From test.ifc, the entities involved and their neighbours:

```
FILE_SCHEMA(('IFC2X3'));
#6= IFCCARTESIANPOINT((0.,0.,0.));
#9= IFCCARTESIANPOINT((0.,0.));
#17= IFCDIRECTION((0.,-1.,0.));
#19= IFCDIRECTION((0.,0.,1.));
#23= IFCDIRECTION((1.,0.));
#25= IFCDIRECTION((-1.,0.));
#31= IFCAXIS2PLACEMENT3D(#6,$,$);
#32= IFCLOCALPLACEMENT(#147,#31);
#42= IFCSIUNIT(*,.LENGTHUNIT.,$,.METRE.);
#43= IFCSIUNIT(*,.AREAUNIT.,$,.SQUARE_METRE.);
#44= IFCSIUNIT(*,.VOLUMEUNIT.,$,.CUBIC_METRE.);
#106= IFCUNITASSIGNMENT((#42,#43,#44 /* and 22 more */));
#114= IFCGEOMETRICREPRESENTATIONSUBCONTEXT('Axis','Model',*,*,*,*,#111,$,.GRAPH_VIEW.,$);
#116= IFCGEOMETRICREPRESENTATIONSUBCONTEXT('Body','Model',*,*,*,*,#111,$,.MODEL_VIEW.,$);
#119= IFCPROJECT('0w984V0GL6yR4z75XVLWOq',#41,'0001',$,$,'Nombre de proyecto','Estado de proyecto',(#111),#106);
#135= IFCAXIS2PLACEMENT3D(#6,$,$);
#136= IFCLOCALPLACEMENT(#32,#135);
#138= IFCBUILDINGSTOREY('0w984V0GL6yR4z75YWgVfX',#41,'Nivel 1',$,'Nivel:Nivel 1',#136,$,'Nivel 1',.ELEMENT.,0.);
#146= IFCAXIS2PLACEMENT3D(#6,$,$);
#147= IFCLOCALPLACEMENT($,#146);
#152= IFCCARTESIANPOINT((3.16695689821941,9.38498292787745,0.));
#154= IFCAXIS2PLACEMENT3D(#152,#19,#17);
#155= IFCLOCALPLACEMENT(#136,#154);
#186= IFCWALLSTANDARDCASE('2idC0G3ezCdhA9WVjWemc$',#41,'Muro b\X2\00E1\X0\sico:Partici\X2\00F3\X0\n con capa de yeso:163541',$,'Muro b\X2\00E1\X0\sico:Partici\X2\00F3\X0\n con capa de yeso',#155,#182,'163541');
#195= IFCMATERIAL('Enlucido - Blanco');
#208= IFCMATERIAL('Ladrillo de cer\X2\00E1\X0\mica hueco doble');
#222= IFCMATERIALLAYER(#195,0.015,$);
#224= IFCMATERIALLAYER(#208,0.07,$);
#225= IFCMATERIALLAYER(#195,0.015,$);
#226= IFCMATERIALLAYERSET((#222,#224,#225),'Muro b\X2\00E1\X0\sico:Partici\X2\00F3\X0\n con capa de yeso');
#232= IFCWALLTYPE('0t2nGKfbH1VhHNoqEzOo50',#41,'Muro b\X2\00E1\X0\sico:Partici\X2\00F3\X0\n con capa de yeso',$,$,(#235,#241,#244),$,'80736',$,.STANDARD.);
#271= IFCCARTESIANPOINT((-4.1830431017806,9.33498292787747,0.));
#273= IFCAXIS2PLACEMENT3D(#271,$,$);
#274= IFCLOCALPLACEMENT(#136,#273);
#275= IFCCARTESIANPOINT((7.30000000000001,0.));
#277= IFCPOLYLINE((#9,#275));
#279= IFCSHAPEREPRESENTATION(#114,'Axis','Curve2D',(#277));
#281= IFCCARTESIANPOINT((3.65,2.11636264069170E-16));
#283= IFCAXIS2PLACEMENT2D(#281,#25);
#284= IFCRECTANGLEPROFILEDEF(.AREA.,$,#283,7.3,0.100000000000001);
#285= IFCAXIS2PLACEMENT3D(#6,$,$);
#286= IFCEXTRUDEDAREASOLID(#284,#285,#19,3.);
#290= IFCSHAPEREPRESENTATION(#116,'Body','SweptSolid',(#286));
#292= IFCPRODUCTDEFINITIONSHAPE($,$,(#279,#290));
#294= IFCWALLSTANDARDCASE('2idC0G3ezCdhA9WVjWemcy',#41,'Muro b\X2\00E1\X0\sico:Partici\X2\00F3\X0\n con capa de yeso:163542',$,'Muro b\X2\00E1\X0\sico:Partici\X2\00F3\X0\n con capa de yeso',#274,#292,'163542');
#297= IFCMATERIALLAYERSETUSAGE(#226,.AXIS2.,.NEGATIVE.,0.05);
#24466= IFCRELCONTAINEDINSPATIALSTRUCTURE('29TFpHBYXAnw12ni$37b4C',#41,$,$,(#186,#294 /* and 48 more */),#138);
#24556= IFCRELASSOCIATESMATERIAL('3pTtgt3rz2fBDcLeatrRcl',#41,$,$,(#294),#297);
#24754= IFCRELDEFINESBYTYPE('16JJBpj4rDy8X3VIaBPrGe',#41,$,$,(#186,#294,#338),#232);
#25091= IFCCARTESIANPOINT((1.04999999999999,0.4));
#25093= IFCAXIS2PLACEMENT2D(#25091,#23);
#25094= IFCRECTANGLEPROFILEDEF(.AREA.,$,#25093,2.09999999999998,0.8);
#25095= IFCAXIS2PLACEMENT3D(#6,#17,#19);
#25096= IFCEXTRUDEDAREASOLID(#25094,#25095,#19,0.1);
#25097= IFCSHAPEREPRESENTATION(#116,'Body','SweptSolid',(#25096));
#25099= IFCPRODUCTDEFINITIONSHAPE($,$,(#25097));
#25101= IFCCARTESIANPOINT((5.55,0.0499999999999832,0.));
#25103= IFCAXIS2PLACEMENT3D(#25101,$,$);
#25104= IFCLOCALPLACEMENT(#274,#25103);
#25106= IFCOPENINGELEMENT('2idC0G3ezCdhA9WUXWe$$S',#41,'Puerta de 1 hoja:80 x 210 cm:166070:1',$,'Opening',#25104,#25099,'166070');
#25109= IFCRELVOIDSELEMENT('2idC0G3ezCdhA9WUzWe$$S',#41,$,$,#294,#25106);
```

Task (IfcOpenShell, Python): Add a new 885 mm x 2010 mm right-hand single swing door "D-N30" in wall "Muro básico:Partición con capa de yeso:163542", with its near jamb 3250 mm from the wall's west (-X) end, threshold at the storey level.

```python
import numpy as np
import ifcopenshell
import ifcopenshell.api.feature
import ifcopenshell.api.geometry
import ifcopenshell.api.root
import ifcopenshell.api.spatial
import ifcopenshell.api.type
import ifcopenshell.geom
import ifcopenshell.util.element
import ifcopenshell.util.placement
import ifcopenshell.util.representation
import ifcopenshell.util.shape
import ifcopenshell.util.unit

model = ifcopenshell.open("test.ifc")
unit_scale = ifcopenshell.util.unit.calculate_unit_scale(model)
settings = ifcopenshell.geom.settings()


def volume(element):
    """Net volume in cubic metres, openings subtracted."""
    shape = ifcopenshell.geom.create_shape(settings, element)
    return ifcopenshell.util.shape.get_volume(shape.geometry)


wall = model.by_id(294)
storey = ifcopenshell.util.element.get_container(wall, ifc_class="IfcBuildingStorey")
context = ifcopenshell.util.representation.get_context(model, "Model", "Body", "MODEL_VIEW")
before = volume(wall)

width, height, from_end, sill = 0.885, 2.01, 3.25, 0.0  # metres

# The wall runs along its own X axis, and the end named is its -X end.
wall_shape = ifcopenshell.geom.create_shape(settings, wall)
x, y, z = ifcopenshell.util.shape.get_vertices(wall_shape.geometry).T
start = x.min() + from_end
face, thickness = float(y.min()), float(y.max() - y.min())
wall_matrix = ifcopenshell.util.placement.get_local_placement(wall.ObjectPlacement)
level = ifcopenshell.util.placement.get_local_placement(storey.ObjectPlacement)[2, 3]


def in_wall(x, y):
    """Placement at x, y metres in the wall's axes, at sill height."""
    matrix = wall_matrix.copy()
    matrix[:, 3] = wall_matrix @ np.array([x / unit_scale, y / unit_scale, 0.0, 1.0])
    matrix[2, 3] = level + sill / unit_scale
    return matrix


# Opening: a box that overshoots both wall faces by 50 mm.
opening = ifcopenshell.api.root.create_entity(model, ifc_class="IfcOpeningElement")
box = ifcopenshell.api.geometry.add_wall_representation(
    model, context=context, length=width, height=height, thickness=thickness + 0.1
)
ifcopenshell.api.geometry.assign_representation(model, product=opening, representation=box)
ifcopenshell.api.geometry.edit_object_placement(model, product=opening, matrix=in_wall(start, face - 0.05), is_si=False)
ifcopenshell.api.feature.add_feature(model, feature=opening, element=wall)

door = ifcopenshell.api.root.create_entity(model, ifc_class="IfcDoor", name="D-N30")
door.OverallWidth, door.OverallHeight = width / unit_scale, height / unit_scale
body = ifcopenshell.api.geometry.add_door_representation(
    model,
    context=context,
    overall_width=door.OverallWidth,
    overall_height=door.OverallHeight,
    operation_type="SINGLE_SWING_RIGHT",
    lining_properties={"LiningDepth": thickness / unit_scale, "ThresholdDepth": thickness / unit_scale},
)
ifcopenshell.api.geometry.assign_representation(model, product=door, representation=body)
ifcopenshell.api.spatial.assign_container(model, products=[door], relating_structure=storey)
fills = ifcopenshell.api.feature.add_filling(model, opening=opening, element=door)
fills.OwnerHistory = door.OwnerHistory  # required in IFC2X3

# IFC2X3 keeps the operation on the door style.
style = ifcopenshell.api.root.create_entity(model, ifc_class="IfcDoorStyle", name="D-N30")
style.OperationType, style.ConstructionType = "SINGLE_SWING_RIGHT", "NOTDEFINED"
style.ParameterTakesPrecedence = style.Sizeable = False
ifcopenshell.api.type.assign_type(model, related_objects=[door], relating_type=style)

# The lining spans the wall, so the door starts at the wall face.
ifcopenshell.api.geometry.edit_object_placement(model, product=door, matrix=in_wall(start, face), is_si=False)

after = volume(wall)

print(f"wall volume {before:.3f} -> {after:.3f} m3")

model.write("test_edited.ifc")
```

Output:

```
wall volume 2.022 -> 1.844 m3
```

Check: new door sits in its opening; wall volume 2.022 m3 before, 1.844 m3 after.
